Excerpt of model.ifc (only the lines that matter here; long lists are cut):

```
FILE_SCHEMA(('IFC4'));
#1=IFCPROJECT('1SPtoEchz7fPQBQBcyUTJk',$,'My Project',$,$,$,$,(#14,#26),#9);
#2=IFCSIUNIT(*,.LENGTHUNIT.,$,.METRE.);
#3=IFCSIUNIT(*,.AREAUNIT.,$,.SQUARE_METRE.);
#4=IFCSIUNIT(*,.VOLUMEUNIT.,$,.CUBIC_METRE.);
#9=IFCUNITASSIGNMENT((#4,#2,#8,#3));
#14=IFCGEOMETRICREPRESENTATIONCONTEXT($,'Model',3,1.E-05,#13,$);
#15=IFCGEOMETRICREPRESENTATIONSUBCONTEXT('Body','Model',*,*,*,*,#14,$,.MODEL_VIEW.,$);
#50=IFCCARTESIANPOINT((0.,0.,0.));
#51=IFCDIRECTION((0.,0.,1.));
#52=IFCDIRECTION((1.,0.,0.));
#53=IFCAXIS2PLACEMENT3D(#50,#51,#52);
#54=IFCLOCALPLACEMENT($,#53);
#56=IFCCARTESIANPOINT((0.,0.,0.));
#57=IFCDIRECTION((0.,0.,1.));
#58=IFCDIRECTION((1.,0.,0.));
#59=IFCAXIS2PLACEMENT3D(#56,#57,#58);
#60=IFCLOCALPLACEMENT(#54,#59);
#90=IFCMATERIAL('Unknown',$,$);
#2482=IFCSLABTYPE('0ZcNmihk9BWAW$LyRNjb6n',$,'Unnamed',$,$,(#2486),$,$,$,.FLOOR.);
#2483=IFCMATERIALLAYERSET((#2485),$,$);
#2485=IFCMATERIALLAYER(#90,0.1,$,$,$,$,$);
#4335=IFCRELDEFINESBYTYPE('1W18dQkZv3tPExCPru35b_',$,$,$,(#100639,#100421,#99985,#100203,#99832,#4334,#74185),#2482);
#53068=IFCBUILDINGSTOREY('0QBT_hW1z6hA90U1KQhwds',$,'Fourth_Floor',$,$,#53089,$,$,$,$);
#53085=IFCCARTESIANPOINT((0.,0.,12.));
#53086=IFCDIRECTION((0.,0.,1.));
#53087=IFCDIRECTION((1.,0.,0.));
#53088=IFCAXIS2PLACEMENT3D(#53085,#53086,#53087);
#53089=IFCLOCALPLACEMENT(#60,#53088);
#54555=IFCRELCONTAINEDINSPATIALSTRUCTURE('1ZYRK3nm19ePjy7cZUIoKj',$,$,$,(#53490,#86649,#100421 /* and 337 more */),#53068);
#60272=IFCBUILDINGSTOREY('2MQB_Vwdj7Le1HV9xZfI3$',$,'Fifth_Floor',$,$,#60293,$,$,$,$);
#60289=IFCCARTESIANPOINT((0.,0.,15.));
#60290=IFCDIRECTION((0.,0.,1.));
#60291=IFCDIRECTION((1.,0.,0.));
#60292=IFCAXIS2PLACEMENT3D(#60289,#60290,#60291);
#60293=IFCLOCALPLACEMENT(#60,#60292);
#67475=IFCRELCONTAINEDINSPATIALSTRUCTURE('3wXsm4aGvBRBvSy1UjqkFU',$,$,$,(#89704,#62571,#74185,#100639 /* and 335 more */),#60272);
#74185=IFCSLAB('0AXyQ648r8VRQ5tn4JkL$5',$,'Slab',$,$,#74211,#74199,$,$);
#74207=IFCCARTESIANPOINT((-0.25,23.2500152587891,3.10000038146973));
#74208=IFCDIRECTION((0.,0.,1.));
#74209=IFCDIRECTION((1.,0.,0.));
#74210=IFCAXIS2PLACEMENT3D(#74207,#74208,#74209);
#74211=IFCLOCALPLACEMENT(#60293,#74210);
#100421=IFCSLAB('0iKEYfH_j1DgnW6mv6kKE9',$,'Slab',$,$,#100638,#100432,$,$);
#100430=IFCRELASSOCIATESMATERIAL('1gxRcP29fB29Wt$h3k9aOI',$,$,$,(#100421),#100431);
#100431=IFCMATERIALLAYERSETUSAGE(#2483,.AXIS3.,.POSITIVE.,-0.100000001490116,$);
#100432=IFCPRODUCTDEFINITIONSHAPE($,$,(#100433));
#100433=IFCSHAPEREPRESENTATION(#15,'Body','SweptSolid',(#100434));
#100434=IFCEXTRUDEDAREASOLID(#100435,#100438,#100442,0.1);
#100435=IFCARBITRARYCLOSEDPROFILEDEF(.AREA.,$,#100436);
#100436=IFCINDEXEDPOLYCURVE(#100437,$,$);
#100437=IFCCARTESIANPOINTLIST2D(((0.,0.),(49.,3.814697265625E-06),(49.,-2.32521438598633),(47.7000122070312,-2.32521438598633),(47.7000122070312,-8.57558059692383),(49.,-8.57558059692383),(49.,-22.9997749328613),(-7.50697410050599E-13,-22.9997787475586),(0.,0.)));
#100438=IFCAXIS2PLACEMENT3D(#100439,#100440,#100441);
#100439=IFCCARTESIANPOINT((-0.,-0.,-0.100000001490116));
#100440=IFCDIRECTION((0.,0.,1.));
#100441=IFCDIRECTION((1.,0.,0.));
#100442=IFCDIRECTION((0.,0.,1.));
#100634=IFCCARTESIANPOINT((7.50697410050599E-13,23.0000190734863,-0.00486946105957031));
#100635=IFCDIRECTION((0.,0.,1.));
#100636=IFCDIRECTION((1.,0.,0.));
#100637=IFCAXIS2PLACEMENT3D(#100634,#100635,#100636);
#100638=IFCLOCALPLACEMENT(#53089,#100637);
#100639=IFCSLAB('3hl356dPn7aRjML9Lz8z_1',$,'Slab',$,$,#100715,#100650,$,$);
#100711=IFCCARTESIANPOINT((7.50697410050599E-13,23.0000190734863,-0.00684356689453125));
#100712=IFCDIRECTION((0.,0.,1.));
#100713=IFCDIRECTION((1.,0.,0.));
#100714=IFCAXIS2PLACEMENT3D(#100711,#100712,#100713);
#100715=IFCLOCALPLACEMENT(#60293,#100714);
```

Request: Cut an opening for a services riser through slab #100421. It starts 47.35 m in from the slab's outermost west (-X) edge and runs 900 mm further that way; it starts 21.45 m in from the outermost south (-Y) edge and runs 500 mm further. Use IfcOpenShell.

```python
import numpy as np
import ifcopenshell
import ifcopenshell.api.feature
import ifcopenshell.api.geometry
import ifcopenshell.api.root
import ifcopenshell.geom
import ifcopenshell.util.placement
import ifcopenshell.util.representation
import ifcopenshell.util.shape
import ifcopenshell.util.unit

model = ifcopenshell.open("model.ifc")
unit_scale = ifcopenshell.util.unit.calculate_unit_scale(model)
settings = ifcopenshell.geom.settings()


def volume(element):
    """Net volume in cubic metres, openings subtracted."""
    shape = ifcopenshell.geom.create_shape(settings, element)
    return ifcopenshell.util.shape.get_volume(shape.geometry)


slab = model.by_guid("0iKEYfH_j1DgnW6mv6kKE9")
before = volume(slab)

# Extent in the slab's own axes, in metres. The edges named are its -X and -Y sides.
slab_shape = ifcopenshell.geom.create_shape(settings, slab)
vertices = ifcopenshell.util.shape.get_vertices(slab_shape.geometry)
x_min, y_min, bottom = vertices.min(axis=0)
top = vertices[:, 2].max()

opening = ifcopenshell.api.root.create_entity(model, ifc_class="IfcOpeningElement", name="Services riser opening", predefined_type="OPENING")
context = ifcopenshell.util.representation.get_context(model, "Model", "Body", "MODEL_VIEW")
width, depth = 0.9, 0.5
outline = [(0.0, 0.0), (width, 0.0), (width, depth), (0.0, depth), (0.0, 0.0)]
# Overshoot both faces by 50 mm so the cut is clean.
shape = ifcopenshell.api.geometry.add_slab_representation(
    model, context=context, depth=top - bottom + 0.1, polyline=outline
)
ifcopenshell.api.geometry.assign_representation(model, product=opening, representation=shape)

matrix = ifcopenshell.util.placement.get_local_placement(slab.ObjectPlacement)
matrix[:, 3] = matrix @ np.append(np.array([x_min + 47.35, y_min + 21.45, bottom - 0.05]) / unit_scale, 1.0)
ifcopenshell.api.geometry.edit_object_placement(model, product=opening, matrix=matrix, is_si=False)
ifcopenshell.api.feature.add_feature(model, feature=opening, element=slab)

after = volume(slab)

print(f"slab volume {before:.3f} -> {after:.3f} m3")

model.write("model_v2.ifc")
```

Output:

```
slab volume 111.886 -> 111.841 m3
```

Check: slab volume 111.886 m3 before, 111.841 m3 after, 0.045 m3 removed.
